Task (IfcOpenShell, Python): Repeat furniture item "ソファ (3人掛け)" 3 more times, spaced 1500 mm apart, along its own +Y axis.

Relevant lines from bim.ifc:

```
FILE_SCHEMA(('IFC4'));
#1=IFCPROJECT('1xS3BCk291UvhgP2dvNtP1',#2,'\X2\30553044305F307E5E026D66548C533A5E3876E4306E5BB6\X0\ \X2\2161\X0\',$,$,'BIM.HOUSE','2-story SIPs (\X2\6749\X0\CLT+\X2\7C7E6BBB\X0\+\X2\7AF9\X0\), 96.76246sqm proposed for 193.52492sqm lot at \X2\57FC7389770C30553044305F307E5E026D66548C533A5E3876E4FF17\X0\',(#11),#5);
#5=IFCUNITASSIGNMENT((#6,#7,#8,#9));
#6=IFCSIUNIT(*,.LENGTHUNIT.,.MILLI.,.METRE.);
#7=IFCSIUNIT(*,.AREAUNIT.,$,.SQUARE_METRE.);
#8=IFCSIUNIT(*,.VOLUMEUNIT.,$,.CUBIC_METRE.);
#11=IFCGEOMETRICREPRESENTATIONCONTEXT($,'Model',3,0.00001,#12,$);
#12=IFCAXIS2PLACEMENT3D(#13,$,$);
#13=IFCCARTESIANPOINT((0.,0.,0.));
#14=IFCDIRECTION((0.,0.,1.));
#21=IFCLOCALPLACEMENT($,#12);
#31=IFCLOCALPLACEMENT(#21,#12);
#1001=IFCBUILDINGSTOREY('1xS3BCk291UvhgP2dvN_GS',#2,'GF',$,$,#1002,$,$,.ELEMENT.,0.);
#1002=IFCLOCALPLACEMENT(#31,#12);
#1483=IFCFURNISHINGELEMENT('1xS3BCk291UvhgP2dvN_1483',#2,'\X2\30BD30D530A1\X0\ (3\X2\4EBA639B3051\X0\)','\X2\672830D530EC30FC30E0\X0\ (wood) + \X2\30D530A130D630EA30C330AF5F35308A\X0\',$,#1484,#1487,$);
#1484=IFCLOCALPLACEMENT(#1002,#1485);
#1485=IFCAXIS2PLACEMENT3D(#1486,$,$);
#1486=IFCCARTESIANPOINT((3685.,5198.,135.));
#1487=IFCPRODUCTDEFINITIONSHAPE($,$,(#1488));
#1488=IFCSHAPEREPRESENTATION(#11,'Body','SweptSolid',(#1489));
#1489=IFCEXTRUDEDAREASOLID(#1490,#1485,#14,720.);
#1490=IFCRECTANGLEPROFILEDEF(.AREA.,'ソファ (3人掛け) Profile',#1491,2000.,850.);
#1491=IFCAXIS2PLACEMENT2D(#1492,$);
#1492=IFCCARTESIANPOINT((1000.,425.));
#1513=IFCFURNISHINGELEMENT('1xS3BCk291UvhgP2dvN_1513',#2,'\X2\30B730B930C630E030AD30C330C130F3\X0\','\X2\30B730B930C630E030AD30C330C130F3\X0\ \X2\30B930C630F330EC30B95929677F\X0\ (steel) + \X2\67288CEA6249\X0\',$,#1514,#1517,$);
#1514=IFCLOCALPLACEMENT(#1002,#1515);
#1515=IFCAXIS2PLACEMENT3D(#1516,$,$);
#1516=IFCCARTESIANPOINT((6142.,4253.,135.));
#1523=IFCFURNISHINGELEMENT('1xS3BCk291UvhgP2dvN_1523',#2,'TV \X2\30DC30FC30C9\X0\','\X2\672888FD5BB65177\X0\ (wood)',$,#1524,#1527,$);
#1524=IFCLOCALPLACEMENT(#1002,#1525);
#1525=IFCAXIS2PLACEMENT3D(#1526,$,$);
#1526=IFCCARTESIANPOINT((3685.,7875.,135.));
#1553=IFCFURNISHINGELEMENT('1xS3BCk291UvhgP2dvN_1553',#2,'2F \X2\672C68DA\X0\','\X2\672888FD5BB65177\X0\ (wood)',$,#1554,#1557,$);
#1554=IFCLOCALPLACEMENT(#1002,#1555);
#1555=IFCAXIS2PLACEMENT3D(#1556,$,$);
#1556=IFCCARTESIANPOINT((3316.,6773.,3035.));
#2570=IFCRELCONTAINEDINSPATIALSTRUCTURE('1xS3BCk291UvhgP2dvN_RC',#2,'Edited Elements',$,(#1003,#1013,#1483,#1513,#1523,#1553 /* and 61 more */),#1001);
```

```python
import ifcopenshell
import ifcopenshell.api.geometry
import ifcopenshell.api.root
import ifcopenshell.util.element
import ifcopenshell.util.placement

model = ifcopenshell.open("bim.ifc")


def reuse_history(source, copy):
    """copy_class also copies each property set's owner history, people and application; keep the originals."""
    for rel in copy.IsDefinedBy:
        if rel.is_a("IfcRelDefinesByProperties") and (history := rel.RelatingPropertyDefinition.OwnerHistory):
            rel.RelatingPropertyDefinition.OwnerHistory = source.OwnerHistory
            ifcopenshell.util.element.remove_deep2(model, history)


source = model.by_guid("1xS3BCk291UvhgP2dvN_1483")
base = ifcopenshell.util.placement.get_local_placement(source.ObjectPlacement)
step = base[:3, 1] * 1500.0

for i in range(1, 4):
    copy = ifcopenshell.api.root.copy_class(model, product=source)
    copy.Representation = ifcopenshell.util.element.copy_deep(
        model, source.Representation, exclude=["IfcGeometricRepresentationContext", "IfcRepresentationMap"]
    )
    reuse_history(source, copy)
    matrix = base.copy()
    matrix[:3, 3] += i * step
    print("added at", matrix[:3, 3].round(3) + 0.0)
    ifcopenshell.api.geometry.edit_object_placement(model, product=copy, matrix=matrix, is_si=False)

model.write("bim_rev.ifc")
```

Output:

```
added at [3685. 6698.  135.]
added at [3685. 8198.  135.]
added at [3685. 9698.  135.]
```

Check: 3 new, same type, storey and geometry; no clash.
